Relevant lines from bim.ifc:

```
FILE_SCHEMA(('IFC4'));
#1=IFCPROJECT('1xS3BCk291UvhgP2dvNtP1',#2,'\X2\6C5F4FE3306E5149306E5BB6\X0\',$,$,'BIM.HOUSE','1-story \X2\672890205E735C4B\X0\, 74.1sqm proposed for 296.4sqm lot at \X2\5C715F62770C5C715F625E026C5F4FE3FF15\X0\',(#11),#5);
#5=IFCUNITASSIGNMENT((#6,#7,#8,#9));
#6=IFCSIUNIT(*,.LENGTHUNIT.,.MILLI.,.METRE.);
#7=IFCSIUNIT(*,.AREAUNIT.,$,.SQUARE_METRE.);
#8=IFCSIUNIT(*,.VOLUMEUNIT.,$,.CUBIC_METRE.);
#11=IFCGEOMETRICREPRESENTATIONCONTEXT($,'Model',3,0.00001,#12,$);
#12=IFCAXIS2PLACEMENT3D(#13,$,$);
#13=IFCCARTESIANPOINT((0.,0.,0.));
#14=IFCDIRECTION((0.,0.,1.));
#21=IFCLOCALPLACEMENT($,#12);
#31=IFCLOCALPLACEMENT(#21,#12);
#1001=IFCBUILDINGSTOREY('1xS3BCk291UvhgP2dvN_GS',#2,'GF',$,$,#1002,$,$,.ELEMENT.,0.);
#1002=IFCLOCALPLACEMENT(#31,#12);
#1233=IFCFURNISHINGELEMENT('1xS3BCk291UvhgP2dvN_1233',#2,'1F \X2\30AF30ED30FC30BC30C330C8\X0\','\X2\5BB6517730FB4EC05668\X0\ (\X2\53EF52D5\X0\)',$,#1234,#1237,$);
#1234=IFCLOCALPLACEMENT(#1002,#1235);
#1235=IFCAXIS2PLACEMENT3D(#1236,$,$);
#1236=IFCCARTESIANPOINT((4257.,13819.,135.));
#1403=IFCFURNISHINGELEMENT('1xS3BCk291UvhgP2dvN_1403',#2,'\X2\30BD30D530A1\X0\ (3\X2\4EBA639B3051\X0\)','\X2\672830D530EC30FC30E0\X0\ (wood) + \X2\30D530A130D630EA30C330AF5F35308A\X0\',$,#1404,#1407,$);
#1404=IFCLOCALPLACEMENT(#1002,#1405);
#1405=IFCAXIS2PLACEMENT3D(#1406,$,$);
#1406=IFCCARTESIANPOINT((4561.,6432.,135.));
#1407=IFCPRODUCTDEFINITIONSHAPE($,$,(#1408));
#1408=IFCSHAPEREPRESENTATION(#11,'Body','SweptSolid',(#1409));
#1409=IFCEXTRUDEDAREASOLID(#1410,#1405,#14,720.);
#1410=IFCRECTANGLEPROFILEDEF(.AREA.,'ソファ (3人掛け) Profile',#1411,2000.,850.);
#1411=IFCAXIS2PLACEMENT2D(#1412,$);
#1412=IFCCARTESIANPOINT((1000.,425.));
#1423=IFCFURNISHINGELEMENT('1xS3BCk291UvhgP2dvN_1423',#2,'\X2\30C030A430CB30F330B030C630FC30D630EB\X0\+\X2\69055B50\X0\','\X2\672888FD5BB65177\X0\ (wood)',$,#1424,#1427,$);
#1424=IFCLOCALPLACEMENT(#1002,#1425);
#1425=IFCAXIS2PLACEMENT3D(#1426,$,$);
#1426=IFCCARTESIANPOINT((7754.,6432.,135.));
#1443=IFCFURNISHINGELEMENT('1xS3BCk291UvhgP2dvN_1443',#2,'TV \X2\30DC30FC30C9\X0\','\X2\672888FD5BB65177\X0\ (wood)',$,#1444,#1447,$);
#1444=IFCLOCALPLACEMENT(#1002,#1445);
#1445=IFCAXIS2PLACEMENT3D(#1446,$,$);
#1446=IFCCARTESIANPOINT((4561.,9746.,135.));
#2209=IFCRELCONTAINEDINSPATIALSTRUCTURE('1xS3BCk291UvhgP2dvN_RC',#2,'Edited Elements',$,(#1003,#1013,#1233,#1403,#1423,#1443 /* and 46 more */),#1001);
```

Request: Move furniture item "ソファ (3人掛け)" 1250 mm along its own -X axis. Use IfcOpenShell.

```python
import ifcopenshell
import ifcopenshell.api.geometry
import ifcopenshell.util.placement
import ifcopenshell.util.unit

model = ifcopenshell.open("bim.ifc")
unit_scale = ifcopenshell.util.unit.calculate_unit_scale(model)

item = model.by_guid("1xS3BCk291UvhgP2dvN_1403")
matrix = ifcopenshell.util.placement.get_local_placement(item.ObjectPlacement)
matrix[:3, 3] -= matrix[:3, 0] * 1.25 / unit_scale
ifcopenshell.api.geometry.edit_object_placement(model, product=item, matrix=matrix, is_si=False)

print(ifcopenshell.util.placement.get_local_placement(item.ObjectPlacement).round(3) + 0.0)

model.write("bim_rev.ifc")
```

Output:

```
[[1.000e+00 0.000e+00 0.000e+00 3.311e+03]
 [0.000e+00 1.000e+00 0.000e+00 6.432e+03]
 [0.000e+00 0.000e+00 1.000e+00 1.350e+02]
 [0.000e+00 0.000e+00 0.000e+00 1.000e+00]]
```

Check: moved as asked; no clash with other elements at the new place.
